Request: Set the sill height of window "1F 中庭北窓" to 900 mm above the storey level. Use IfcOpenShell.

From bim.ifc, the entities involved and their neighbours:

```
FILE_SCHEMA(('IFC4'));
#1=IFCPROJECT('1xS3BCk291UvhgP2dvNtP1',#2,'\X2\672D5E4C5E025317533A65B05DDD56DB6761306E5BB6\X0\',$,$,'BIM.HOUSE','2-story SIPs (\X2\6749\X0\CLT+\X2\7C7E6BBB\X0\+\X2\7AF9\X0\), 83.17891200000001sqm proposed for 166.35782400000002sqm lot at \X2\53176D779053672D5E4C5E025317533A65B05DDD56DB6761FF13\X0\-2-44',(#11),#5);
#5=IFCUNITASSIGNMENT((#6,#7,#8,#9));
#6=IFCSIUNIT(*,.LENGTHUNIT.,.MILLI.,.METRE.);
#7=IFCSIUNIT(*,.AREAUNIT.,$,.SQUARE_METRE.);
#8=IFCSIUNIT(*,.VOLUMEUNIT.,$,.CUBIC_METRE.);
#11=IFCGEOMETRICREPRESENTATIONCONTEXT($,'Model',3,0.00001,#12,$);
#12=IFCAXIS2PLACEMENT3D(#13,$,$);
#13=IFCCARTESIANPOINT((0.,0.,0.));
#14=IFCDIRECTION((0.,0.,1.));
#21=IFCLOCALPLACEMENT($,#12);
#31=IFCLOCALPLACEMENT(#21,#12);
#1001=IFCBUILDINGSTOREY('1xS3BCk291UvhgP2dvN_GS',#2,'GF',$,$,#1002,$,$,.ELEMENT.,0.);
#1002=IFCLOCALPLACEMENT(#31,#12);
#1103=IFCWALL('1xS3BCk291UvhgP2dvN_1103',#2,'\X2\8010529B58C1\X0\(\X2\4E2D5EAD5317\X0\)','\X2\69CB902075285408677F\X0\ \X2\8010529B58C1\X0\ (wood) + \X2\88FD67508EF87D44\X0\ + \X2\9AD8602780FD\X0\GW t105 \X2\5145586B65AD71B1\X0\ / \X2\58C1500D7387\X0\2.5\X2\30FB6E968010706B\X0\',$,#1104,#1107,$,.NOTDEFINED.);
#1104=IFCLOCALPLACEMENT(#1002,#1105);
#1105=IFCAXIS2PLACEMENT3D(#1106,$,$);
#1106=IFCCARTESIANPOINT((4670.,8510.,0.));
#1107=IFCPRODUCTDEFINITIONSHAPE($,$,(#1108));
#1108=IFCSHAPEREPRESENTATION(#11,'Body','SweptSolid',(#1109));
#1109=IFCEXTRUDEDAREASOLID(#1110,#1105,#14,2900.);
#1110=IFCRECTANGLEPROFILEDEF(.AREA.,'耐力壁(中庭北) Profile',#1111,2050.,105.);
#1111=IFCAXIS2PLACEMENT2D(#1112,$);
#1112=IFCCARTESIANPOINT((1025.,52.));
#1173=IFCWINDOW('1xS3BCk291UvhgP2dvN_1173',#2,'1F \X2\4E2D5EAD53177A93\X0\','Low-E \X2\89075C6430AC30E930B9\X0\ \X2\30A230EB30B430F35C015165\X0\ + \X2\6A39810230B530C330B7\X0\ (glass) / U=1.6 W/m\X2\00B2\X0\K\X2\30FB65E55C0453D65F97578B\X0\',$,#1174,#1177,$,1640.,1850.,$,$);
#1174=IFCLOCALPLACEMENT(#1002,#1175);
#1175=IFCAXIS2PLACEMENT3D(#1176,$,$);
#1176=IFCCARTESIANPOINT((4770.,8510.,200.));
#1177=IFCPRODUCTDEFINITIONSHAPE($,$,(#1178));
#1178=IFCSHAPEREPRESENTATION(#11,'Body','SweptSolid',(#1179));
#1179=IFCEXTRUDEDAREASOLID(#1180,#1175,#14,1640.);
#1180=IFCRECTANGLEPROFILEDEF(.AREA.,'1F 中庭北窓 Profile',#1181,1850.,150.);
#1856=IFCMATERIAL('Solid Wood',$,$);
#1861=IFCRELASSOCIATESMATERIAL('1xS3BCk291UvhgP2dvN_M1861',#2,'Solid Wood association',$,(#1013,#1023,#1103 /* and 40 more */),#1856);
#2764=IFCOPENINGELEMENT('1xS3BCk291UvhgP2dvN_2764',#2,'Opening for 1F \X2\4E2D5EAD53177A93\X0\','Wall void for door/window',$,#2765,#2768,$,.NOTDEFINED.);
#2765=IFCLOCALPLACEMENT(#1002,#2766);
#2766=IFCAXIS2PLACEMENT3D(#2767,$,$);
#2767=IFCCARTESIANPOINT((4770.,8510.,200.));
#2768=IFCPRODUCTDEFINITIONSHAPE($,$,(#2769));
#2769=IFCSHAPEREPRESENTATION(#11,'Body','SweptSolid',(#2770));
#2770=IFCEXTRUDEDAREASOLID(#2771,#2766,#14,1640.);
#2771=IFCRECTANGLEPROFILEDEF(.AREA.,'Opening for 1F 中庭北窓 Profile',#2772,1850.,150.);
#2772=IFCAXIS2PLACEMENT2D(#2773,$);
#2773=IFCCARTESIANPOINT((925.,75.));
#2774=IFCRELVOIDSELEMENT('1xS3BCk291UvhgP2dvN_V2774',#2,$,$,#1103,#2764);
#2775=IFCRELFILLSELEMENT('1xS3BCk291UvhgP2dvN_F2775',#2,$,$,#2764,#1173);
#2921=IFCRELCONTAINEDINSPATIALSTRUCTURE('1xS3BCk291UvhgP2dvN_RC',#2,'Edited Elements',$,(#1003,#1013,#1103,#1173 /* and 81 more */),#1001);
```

```python
import numpy as np
import ifcopenshell
import ifcopenshell.api.geometry
import ifcopenshell.geom
import ifcopenshell.util.element
import ifcopenshell.util.placement
import ifcopenshell.util.shape
import ifcopenshell.util.unit

model = ifcopenshell.open("bim.ifc")
unit_scale = ifcopenshell.util.unit.calculate_unit_scale(model)

window = model.by_guid("1xS3BCk291UvhgP2dvN_1173")
opening = window.FillsVoids[0].RelatingOpeningElement
storey = ifcopenshell.util.element.get_container(window, ifc_class="IfcBuildingStorey")
level = ifcopenshell.util.placement.get_local_placement(storey.ObjectPlacement)[2, 3]

# The opening's origin need not be at the sill, so measure its lowest point.
shape = ifcopenshell.geom.create_shape(ifcopenshell.geom.settings(), opening)
bottom = ifcopenshell.util.shape.get_shape_bottom_elevation(shape, shape.geometry) / unit_scale
dz = level + 0.9 / unit_scale - bottom

shift = np.array([0.0, 0.0, dz])
# The window is not placed relative to its opening, so move both.
for product in (opening, window):
    matrix = ifcopenshell.util.placement.get_local_placement(product.ObjectPlacement)
    matrix[:3, 3] += shift
    ifcopenshell.api.geometry.edit_object_placement(model, product=product, matrix=matrix, is_si=False)

print(f"moved by {dz * unit_scale:+.3f} m")

model.write("bim_v2.ifc")
```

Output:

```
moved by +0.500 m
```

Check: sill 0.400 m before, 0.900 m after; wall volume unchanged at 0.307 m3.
